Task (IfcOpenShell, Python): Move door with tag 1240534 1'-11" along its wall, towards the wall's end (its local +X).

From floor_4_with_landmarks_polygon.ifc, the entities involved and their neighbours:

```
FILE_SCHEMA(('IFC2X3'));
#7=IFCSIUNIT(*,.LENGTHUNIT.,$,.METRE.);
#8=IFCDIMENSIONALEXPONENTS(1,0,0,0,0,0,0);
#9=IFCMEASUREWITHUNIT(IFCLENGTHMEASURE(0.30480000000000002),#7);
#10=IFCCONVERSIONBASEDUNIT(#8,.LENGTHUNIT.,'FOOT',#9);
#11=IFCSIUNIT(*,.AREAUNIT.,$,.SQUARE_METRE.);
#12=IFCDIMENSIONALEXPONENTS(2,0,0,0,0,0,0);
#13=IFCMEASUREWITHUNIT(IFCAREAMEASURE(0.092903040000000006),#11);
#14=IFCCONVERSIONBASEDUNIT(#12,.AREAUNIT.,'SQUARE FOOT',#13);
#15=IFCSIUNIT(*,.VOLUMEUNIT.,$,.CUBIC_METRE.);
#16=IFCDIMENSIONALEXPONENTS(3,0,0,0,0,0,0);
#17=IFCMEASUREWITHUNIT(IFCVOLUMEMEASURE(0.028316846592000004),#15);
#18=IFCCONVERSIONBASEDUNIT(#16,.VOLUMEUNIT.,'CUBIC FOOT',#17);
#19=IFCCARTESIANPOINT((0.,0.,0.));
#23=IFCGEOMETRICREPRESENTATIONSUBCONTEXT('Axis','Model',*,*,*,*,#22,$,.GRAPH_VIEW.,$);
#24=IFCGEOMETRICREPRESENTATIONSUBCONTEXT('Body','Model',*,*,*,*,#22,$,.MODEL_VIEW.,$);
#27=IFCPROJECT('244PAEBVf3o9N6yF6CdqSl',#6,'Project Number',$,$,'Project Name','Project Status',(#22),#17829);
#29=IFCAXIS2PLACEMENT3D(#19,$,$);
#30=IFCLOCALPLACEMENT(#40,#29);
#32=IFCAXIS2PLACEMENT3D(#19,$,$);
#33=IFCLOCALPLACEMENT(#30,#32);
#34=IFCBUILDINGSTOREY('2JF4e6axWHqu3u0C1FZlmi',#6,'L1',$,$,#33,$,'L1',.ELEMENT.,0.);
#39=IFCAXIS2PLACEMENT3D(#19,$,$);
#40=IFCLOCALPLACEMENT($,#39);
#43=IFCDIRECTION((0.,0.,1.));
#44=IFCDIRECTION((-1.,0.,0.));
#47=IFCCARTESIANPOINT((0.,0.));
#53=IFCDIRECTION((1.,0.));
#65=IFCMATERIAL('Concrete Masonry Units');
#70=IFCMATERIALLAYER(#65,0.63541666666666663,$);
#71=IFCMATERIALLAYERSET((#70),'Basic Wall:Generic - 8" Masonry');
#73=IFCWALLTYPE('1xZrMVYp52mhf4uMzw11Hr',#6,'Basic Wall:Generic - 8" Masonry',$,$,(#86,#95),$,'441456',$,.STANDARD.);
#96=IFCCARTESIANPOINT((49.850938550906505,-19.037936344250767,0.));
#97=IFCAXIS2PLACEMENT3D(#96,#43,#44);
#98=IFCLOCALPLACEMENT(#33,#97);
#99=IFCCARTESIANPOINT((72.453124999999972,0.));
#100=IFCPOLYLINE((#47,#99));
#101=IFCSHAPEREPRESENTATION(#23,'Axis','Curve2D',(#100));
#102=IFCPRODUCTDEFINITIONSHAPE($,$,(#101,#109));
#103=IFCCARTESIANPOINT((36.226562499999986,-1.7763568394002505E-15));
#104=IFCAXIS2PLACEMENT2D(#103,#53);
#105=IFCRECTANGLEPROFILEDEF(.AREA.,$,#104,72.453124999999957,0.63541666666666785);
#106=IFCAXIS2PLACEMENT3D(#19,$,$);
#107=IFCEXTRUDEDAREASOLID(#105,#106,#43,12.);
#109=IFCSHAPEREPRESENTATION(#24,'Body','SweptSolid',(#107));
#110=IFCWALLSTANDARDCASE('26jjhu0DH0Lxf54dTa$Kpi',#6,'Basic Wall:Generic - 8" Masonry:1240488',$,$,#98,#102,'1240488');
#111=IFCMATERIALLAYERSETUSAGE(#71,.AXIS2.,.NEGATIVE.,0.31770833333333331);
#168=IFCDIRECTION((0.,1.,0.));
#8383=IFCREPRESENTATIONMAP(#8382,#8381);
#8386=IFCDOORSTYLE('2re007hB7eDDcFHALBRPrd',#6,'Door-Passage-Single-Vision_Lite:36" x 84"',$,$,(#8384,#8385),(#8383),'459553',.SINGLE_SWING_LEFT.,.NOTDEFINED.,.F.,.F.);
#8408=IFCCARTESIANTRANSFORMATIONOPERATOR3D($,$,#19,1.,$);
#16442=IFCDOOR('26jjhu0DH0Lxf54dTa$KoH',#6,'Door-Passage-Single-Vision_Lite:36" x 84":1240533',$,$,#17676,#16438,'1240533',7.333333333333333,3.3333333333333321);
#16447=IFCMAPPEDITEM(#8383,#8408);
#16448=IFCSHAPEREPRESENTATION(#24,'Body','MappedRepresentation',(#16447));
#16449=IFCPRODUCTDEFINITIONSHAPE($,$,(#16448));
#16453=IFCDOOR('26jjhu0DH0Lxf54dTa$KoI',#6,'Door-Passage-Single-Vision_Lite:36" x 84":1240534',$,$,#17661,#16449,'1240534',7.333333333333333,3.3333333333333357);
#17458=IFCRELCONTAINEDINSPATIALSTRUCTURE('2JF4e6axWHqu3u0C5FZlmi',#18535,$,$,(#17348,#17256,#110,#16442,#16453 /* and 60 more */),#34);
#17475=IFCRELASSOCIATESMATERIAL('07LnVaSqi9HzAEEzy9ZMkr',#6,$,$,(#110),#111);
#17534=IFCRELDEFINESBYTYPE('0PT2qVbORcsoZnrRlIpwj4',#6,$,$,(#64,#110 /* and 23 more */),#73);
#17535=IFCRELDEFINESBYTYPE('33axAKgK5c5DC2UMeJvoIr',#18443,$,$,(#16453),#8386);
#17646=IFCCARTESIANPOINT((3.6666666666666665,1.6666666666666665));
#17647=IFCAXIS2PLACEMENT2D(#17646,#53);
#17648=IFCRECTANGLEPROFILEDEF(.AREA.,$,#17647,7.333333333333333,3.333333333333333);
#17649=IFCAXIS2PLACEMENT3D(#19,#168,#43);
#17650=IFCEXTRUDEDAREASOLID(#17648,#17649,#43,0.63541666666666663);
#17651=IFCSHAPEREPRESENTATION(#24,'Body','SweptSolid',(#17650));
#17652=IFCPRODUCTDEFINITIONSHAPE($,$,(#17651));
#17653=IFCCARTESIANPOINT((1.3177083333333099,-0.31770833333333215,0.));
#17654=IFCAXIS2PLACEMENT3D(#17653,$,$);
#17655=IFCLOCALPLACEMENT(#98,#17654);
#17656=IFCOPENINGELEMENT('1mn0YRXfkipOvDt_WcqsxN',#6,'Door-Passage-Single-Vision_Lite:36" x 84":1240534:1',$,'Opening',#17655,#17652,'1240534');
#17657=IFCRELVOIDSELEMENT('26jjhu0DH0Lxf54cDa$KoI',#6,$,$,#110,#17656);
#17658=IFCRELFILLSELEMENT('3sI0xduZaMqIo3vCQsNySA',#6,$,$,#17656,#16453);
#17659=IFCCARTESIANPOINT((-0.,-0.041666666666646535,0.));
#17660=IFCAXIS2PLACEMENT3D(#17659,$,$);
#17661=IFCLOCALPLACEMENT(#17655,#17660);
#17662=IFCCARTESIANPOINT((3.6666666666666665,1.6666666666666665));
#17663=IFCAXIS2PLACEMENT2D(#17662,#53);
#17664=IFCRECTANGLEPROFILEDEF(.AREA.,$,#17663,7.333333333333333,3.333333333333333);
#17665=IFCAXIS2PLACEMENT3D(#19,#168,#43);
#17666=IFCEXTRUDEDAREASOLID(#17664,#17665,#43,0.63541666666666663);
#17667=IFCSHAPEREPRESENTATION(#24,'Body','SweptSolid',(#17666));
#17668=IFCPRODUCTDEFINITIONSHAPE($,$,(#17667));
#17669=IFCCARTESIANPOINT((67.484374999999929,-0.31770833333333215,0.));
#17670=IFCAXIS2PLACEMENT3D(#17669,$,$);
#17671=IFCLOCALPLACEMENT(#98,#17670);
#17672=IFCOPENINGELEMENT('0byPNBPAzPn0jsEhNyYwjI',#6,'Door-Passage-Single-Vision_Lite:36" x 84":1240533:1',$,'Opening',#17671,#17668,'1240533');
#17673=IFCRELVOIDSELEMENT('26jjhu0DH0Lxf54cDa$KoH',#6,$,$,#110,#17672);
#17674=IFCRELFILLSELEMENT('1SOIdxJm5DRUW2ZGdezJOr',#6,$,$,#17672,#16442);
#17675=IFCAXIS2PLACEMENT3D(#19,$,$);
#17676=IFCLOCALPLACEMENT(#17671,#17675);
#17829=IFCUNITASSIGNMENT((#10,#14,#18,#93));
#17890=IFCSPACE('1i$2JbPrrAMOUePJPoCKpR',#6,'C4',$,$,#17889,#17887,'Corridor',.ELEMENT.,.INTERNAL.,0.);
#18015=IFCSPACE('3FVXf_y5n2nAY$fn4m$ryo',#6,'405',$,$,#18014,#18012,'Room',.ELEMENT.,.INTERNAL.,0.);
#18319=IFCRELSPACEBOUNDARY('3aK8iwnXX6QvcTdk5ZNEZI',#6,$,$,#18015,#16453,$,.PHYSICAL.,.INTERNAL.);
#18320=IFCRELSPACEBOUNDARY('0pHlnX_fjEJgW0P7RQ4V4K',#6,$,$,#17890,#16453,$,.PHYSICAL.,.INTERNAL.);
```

```python
import ifcopenshell
import ifcopenshell.api.geometry
import ifcopenshell.util.placement
import ifcopenshell.util.unit

model = ifcopenshell.open("floor_4_with_landmarks_polygon.ifc")
unit_scale = ifcopenshell.util.unit.calculate_unit_scale(model)

door = model.by_guid("26jjhu0DH0Lxf54dTa$KoI")
opening = door.FillsVoids[0].RelatingOpeningElement
wall = opening.VoidsElements[0].RelatingBuildingElement

wall_matrix = ifcopenshell.util.placement.get_local_placement(wall.ObjectPlacement)
shift = wall_matrix[:3, 0] * 23 * 0.0254 / unit_scale
before = ifcopenshell.util.placement.get_local_placement(door.ObjectPlacement)[:3, 3].copy()

# The door is placed relative to its opening, so it follows when the opening moves.
matrix = ifcopenshell.util.placement.get_local_placement(opening.ObjectPlacement)
matrix[:3, 3] += shift
ifcopenshell.api.geometry.edit_object_placement(
    model, product=opening, matrix=matrix, is_si=False, should_transform_children=True
)

after = ifcopenshell.util.placement.get_local_placement(door.ObjectPlacement)[:3, 3]
print("door moved by", (after - before).round(3) + 0.0)

model.write("floor_4_with_landmarks_polygon_v2.ifc")
```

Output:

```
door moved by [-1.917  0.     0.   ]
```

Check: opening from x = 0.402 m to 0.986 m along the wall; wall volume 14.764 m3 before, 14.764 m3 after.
